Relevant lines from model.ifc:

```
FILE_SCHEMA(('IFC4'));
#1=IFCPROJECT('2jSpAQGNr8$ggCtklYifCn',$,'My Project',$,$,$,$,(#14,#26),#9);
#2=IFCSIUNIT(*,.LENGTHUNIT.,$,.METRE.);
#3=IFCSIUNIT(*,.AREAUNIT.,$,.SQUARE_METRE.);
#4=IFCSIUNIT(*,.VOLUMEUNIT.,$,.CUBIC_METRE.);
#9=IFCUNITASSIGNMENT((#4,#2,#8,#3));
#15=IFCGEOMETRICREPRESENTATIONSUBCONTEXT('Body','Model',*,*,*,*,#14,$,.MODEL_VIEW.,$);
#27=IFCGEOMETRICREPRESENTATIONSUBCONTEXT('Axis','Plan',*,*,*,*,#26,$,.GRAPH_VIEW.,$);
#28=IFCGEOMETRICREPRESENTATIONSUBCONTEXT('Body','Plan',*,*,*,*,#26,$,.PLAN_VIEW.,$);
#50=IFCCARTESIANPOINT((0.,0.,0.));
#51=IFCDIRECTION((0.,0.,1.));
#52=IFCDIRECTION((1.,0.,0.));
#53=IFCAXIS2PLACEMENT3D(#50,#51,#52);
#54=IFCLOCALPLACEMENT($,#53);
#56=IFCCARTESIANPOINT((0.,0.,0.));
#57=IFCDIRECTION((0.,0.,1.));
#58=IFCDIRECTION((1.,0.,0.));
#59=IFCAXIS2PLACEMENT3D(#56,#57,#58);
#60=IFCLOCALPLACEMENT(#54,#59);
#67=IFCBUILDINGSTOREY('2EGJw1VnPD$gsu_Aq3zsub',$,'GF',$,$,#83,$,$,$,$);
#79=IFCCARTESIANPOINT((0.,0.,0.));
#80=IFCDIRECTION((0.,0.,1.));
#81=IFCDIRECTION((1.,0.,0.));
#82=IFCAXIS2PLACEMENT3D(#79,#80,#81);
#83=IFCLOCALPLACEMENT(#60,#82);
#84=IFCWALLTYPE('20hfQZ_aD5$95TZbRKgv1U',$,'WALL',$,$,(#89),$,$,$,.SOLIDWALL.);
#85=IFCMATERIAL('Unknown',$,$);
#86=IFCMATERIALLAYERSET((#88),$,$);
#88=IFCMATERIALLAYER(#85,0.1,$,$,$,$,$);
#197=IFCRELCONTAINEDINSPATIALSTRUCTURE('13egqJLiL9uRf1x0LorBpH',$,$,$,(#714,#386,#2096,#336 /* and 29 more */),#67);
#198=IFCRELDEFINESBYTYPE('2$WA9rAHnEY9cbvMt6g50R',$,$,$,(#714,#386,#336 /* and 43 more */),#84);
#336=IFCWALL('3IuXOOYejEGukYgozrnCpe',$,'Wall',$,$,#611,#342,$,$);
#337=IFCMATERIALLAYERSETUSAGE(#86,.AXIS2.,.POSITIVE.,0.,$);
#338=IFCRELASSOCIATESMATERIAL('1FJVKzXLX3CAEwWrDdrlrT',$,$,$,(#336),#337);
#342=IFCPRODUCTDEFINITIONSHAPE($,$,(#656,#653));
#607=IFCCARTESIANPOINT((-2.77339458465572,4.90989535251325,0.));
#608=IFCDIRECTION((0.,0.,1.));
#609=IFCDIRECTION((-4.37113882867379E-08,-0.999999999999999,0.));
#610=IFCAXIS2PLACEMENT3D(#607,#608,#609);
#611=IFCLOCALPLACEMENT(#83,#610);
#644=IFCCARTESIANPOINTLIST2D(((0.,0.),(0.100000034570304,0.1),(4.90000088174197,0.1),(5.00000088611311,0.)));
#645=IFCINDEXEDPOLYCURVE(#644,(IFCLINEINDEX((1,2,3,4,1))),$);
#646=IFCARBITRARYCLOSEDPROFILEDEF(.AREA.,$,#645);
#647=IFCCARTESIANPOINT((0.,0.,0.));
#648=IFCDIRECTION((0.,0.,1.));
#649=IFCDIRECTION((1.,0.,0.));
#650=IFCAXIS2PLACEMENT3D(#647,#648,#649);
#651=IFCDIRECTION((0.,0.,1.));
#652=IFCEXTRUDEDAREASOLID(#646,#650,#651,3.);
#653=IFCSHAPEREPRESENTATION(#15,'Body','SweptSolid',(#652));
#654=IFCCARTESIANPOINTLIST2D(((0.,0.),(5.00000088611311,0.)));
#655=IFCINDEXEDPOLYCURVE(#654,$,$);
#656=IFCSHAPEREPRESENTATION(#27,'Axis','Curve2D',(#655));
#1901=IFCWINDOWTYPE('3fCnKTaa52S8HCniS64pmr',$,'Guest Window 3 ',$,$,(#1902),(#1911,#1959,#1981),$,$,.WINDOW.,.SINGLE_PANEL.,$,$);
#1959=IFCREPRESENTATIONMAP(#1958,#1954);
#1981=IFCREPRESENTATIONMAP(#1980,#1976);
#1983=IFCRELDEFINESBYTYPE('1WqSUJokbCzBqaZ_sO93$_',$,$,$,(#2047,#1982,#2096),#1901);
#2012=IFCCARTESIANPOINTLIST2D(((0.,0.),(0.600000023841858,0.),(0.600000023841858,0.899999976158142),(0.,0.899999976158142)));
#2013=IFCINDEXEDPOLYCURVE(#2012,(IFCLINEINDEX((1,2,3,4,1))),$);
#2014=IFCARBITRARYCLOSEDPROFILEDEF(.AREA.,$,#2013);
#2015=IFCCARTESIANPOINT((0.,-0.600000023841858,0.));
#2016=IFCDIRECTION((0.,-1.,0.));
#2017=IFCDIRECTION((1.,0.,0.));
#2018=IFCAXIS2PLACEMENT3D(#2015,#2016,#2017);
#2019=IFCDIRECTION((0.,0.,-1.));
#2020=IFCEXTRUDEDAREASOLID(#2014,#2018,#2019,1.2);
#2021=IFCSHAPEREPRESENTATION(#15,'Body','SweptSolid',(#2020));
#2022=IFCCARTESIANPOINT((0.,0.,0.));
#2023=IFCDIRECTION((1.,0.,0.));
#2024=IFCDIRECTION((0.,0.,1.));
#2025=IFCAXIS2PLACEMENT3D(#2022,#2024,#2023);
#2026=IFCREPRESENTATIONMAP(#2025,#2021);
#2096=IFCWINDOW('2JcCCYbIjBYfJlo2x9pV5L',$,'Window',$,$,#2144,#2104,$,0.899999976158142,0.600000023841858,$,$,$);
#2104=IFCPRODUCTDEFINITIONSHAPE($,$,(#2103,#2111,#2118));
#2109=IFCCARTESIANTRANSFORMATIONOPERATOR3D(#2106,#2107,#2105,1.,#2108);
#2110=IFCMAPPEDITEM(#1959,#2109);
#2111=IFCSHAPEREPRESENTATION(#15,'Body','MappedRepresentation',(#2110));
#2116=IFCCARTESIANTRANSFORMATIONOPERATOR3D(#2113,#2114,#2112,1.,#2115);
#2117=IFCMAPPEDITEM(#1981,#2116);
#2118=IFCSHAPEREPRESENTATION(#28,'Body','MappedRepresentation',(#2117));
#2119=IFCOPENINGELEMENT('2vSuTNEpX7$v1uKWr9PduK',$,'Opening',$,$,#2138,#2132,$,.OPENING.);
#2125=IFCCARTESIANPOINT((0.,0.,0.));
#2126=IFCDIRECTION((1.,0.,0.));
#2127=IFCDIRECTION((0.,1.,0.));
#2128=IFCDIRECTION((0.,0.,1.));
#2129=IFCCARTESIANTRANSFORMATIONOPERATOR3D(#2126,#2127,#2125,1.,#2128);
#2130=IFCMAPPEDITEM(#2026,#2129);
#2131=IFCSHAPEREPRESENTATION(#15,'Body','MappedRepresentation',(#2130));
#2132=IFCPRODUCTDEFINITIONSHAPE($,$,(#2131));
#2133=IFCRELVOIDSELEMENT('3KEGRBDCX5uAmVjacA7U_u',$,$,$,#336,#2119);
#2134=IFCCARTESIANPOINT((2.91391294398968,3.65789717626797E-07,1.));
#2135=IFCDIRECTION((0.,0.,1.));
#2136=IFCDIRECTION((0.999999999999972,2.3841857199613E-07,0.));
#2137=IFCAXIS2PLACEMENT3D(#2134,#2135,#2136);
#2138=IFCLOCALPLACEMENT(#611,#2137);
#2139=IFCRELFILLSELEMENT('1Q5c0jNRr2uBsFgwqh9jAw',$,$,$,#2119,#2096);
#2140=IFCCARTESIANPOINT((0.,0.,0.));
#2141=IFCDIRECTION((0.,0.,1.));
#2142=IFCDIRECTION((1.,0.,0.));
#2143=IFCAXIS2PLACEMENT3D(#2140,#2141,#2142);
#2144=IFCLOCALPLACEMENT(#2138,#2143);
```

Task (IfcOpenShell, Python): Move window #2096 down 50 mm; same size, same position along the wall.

```python
import numpy as np
import ifcopenshell
import ifcopenshell.api.geometry
import ifcopenshell.util.placement
import ifcopenshell.util.unit

model = ifcopenshell.open("model.ifc")
unit_scale = ifcopenshell.util.unit.calculate_unit_scale(model)

window = model.by_guid("2JcCCYbIjBYfJlo2x9pV5L")
opening = window.FillsVoids[0].RelatingOpeningElement
dz = -0.05 / unit_scale

shift = np.array([0.0, 0.0, dz])
# The window is placed relative to its opening, so it follows when the opening moves.
matrix = ifcopenshell.util.placement.get_local_placement(opening.ObjectPlacement)
matrix[:3, 3] += shift
ifcopenshell.api.geometry.edit_object_placement(
    model, product=opening, matrix=matrix, is_si=False, should_transform_children=True
)

print(f"moved by {dz * unit_scale:+.3f} m")

model.write("model_edited.ifc")
```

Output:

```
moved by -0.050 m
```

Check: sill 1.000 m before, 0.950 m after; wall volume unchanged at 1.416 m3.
